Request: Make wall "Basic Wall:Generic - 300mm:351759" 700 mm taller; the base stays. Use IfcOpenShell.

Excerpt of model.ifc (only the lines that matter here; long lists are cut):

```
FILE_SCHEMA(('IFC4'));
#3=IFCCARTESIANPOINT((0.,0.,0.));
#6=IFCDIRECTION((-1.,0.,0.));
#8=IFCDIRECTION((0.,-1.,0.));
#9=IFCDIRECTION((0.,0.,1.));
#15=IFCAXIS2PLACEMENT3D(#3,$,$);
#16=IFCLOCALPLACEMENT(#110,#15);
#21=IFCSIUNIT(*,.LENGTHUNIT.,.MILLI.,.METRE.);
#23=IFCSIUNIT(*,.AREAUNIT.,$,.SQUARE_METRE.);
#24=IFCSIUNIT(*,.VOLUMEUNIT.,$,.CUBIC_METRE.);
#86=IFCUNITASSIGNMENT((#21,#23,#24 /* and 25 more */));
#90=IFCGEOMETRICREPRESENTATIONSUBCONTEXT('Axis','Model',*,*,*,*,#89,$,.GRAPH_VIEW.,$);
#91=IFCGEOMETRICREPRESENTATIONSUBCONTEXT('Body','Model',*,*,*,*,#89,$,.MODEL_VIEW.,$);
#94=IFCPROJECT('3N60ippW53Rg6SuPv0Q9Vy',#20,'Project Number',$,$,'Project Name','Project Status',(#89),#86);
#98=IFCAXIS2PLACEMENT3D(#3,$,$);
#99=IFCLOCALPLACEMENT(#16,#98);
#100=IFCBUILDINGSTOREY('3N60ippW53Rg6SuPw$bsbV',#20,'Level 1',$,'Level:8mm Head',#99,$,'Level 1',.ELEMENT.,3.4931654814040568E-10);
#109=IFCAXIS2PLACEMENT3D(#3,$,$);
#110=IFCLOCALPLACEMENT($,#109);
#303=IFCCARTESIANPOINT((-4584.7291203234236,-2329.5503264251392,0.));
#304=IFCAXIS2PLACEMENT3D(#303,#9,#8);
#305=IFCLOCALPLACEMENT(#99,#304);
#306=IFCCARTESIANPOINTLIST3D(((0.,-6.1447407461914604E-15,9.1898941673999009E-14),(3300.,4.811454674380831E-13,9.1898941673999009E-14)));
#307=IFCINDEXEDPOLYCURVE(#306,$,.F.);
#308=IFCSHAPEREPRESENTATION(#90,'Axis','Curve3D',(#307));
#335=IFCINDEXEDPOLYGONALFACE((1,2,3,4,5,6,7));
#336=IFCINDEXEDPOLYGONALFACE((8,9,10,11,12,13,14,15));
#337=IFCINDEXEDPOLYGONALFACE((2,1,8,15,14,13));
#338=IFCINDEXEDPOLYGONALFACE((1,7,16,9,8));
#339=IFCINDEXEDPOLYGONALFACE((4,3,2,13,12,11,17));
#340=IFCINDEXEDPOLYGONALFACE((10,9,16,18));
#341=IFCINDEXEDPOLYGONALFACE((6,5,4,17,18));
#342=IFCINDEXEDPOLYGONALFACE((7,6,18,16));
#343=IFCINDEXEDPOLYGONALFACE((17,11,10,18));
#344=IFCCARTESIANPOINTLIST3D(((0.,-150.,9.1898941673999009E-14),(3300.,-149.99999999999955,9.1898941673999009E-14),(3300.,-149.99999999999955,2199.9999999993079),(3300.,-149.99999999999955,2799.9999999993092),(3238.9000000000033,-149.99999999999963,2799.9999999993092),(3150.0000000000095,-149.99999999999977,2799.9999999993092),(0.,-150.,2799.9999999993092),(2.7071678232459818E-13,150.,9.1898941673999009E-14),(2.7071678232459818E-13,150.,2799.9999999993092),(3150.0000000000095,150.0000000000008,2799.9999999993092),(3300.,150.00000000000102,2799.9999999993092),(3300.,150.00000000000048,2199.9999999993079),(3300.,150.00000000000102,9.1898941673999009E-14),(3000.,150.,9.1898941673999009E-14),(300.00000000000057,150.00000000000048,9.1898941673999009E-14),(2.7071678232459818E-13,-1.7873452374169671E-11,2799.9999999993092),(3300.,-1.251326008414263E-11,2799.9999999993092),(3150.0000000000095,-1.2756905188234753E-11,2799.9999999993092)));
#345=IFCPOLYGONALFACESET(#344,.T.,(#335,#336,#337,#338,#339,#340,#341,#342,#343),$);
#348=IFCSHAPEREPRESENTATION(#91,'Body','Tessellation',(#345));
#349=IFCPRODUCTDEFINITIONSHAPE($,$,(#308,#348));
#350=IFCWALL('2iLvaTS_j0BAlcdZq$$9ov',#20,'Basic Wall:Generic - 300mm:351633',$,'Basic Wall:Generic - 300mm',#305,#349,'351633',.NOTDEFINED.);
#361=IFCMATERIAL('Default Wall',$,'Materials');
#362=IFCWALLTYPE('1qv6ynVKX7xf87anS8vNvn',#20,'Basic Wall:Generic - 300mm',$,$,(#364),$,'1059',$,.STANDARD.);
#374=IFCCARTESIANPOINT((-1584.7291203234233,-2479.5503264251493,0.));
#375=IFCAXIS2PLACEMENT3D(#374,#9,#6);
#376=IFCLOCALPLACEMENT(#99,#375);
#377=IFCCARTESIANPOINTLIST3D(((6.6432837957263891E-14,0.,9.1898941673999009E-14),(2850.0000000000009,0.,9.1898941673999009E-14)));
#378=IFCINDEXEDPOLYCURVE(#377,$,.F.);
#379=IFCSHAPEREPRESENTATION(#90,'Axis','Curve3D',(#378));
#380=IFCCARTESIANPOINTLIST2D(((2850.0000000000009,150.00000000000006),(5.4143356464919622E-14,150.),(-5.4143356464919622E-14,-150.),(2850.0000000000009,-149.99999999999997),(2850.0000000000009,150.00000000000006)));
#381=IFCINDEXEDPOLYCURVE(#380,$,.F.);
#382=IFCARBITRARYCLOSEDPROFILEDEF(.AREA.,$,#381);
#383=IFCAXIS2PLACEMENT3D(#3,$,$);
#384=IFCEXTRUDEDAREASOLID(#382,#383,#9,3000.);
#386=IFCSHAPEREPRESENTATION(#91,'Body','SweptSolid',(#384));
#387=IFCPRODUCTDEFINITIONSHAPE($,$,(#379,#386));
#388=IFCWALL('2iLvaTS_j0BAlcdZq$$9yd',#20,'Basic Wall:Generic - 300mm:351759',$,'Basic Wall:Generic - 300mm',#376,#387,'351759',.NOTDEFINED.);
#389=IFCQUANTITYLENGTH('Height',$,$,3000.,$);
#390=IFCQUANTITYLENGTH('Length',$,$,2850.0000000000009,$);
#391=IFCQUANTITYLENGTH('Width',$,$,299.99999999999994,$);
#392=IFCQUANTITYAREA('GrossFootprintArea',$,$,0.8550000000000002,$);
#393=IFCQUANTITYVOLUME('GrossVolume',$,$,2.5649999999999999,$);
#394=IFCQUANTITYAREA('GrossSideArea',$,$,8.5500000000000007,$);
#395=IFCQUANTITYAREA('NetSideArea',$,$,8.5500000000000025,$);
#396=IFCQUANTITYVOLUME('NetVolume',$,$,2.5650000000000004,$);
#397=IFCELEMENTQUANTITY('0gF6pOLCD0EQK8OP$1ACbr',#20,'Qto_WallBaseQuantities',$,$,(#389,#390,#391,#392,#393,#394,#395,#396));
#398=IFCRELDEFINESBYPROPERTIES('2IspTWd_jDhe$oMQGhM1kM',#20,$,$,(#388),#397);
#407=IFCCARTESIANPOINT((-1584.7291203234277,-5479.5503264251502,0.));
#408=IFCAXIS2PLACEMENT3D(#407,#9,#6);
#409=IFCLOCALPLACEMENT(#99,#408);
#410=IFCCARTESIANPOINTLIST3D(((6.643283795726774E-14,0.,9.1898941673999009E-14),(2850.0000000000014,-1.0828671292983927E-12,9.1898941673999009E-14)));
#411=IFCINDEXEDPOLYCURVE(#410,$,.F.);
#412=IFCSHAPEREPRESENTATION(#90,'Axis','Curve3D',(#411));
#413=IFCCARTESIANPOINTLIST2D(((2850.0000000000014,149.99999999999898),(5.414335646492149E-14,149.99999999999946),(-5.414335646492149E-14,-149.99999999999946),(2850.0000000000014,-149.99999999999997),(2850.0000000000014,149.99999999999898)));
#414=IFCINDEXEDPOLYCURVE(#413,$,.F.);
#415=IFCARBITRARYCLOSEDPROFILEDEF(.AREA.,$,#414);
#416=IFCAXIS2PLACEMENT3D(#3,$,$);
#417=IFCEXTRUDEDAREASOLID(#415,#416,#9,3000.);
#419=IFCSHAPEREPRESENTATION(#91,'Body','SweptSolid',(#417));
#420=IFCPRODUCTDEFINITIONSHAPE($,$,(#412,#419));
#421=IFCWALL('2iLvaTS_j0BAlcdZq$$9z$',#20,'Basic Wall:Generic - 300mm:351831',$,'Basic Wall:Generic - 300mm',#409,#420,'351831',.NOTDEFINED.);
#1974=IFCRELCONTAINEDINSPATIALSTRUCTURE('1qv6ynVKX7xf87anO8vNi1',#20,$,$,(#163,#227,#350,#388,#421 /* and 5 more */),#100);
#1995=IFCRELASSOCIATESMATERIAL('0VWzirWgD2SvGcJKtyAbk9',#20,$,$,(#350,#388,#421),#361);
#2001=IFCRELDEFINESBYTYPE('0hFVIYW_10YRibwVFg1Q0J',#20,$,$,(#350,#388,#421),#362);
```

```python
import ifcopenshell
import ifcopenshell.api.pset
import ifcopenshell.geom
import ifcopenshell.util.element
import ifcopenshell.util.representation
import ifcopenshell.util.shape
import ifcopenshell.util.unit

model = ifcopenshell.open("model.ifc")
unit_scale = ifcopenshell.util.unit.calculate_unit_scale(model)
area_scale = ifcopenshell.util.unit.calculate_unit_scale(model, "AREAUNIT")
volume_scale = ifcopenshell.util.unit.calculate_unit_scale(model, "VOLUMEUNIT")
settings = ifcopenshell.geom.settings()


def volume(element):
    """Net volume in cubic metres, openings subtracted."""
    shape = ifcopenshell.geom.create_shape(settings, element)
    return ifcopenshell.util.shape.get_volume(shape.geometry)


wall = model.by_guid("2iLvaTS_j0BAlcdZq$$9yd")
before = volume(wall)

body = ifcopenshell.util.representation.get_representation(wall, "Model", "Body")
solid = body.Items[0]
old_height = solid.Depth
solid.Depth += 0.7 / unit_scale
after = volume(wall)
thickness = 0.3  # wall thickness in metres

# Update the stored height, areas and volumes.
qto = model.by_id(ifcopenshell.util.element.get_pset(wall, "Qto_WallBaseQuantities", should_inherit=False)["id"])
ifcopenshell.api.pset.edit_qto(model, qto=qto, properties={
    "Height": solid.Depth,
    "GrossVolume": ifcopenshell.util.element.get_pset(wall, "Qto_WallBaseQuantities", "GrossVolume") * solid.Depth / old_height,
    "GrossSideArea": ifcopenshell.util.element.get_pset(wall, "Qto_WallBaseQuantities", "GrossSideArea") * solid.Depth / old_height,
    "NetSideArea": after / thickness / area_scale,
    "NetVolume": after / volume_scale,
})

print(f"height {old_height:g} -> {solid.Depth:g}, volume {before:.3f} -> {after:.3f} m3")

model.write("model_rev.ifc")
```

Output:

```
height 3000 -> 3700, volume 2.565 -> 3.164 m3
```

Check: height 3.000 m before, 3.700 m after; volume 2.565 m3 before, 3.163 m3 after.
